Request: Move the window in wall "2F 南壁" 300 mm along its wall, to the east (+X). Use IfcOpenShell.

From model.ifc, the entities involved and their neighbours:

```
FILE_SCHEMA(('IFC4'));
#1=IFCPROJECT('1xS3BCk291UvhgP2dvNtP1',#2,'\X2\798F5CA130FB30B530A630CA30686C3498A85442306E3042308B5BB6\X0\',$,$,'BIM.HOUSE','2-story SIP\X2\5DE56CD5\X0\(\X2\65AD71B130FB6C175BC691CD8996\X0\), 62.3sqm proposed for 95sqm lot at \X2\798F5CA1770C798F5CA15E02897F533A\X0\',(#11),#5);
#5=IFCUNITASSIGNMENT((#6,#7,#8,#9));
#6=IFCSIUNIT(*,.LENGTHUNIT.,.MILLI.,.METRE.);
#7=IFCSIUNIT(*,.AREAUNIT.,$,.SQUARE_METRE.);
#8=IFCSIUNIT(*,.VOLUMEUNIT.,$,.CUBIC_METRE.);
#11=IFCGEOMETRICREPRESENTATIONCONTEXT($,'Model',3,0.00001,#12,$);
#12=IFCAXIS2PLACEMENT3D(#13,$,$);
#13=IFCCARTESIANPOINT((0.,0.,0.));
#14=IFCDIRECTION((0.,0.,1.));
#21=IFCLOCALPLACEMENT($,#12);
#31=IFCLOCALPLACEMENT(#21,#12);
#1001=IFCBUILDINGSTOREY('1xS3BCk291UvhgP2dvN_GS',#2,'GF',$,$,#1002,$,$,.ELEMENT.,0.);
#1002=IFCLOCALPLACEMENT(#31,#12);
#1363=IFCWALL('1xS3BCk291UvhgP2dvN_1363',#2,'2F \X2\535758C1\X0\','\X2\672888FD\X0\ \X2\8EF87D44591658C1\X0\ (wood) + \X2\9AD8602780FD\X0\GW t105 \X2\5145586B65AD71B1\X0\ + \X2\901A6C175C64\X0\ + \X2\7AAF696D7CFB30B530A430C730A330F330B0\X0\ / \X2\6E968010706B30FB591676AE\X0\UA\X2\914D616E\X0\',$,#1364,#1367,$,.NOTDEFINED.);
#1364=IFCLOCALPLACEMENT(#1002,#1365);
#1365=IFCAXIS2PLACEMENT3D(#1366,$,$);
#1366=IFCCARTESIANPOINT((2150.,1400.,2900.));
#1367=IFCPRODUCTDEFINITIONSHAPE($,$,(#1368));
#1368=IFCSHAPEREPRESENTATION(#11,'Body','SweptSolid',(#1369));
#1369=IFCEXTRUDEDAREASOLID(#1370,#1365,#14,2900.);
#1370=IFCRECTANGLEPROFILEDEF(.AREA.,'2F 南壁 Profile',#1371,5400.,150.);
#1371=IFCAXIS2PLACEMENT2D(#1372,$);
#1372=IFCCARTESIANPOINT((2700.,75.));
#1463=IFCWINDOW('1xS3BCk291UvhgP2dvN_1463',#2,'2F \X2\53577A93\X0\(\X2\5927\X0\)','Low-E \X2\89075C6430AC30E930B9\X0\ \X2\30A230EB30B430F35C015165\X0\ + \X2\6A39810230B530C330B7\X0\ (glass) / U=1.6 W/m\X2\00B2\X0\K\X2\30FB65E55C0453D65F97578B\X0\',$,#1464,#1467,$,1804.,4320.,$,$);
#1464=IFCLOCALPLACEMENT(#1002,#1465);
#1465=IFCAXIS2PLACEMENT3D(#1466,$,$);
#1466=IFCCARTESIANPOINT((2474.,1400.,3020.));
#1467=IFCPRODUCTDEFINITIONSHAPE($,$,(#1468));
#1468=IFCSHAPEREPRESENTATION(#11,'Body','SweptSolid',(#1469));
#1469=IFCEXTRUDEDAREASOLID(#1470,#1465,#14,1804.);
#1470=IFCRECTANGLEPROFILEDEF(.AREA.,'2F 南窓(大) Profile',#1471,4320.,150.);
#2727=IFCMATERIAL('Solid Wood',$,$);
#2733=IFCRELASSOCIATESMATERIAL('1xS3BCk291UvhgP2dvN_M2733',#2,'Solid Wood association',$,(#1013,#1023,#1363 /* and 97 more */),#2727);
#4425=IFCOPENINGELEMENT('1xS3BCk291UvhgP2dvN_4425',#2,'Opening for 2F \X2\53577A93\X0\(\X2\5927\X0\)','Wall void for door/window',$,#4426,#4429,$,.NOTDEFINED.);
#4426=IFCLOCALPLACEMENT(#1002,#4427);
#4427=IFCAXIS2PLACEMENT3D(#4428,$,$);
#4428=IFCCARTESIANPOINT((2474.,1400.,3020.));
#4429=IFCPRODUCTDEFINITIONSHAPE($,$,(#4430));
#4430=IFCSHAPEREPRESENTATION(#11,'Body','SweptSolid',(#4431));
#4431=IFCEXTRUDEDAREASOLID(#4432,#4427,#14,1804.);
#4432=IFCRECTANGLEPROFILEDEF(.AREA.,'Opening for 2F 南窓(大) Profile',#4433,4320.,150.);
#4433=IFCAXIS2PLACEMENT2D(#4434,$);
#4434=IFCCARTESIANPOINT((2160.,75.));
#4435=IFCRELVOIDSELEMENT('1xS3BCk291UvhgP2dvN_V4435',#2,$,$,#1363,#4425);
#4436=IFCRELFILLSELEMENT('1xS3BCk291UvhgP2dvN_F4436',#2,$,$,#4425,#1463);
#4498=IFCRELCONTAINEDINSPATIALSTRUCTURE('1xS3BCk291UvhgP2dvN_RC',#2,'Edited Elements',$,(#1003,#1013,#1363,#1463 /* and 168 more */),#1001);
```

```python
import ifcopenshell
import ifcopenshell.api.geometry
import ifcopenshell.util.placement
import ifcopenshell.util.unit

model = ifcopenshell.open("model.ifc")
unit_scale = ifcopenshell.util.unit.calculate_unit_scale(model)

window = model.by_guid("1xS3BCk291UvhgP2dvN_1463")
opening = window.FillsVoids[0].RelatingOpeningElement
wall = opening.VoidsElements[0].RelatingBuildingElement

wall_matrix = ifcopenshell.util.placement.get_local_placement(wall.ObjectPlacement)
shift = wall_matrix[:3, 0] * 0.3 / unit_scale
before = ifcopenshell.util.placement.get_local_placement(window.ObjectPlacement)[:3, 3].copy()

# The window is not placed relative to its opening, so move both.
for product in (opening, window):
    matrix = ifcopenshell.util.placement.get_local_placement(product.ObjectPlacement)
    matrix[:3, 3] += shift
    ifcopenshell.api.geometry.edit_object_placement(model, product=product, matrix=matrix, is_si=False)

after = ifcopenshell.util.placement.get_local_placement(window.ObjectPlacement)[:3, 3]
print("window moved by", (after - before).round(3) + 0.0)

model.write("model-out.ifc")
```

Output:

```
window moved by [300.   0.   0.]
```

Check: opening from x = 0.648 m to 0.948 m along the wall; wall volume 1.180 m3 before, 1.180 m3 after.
